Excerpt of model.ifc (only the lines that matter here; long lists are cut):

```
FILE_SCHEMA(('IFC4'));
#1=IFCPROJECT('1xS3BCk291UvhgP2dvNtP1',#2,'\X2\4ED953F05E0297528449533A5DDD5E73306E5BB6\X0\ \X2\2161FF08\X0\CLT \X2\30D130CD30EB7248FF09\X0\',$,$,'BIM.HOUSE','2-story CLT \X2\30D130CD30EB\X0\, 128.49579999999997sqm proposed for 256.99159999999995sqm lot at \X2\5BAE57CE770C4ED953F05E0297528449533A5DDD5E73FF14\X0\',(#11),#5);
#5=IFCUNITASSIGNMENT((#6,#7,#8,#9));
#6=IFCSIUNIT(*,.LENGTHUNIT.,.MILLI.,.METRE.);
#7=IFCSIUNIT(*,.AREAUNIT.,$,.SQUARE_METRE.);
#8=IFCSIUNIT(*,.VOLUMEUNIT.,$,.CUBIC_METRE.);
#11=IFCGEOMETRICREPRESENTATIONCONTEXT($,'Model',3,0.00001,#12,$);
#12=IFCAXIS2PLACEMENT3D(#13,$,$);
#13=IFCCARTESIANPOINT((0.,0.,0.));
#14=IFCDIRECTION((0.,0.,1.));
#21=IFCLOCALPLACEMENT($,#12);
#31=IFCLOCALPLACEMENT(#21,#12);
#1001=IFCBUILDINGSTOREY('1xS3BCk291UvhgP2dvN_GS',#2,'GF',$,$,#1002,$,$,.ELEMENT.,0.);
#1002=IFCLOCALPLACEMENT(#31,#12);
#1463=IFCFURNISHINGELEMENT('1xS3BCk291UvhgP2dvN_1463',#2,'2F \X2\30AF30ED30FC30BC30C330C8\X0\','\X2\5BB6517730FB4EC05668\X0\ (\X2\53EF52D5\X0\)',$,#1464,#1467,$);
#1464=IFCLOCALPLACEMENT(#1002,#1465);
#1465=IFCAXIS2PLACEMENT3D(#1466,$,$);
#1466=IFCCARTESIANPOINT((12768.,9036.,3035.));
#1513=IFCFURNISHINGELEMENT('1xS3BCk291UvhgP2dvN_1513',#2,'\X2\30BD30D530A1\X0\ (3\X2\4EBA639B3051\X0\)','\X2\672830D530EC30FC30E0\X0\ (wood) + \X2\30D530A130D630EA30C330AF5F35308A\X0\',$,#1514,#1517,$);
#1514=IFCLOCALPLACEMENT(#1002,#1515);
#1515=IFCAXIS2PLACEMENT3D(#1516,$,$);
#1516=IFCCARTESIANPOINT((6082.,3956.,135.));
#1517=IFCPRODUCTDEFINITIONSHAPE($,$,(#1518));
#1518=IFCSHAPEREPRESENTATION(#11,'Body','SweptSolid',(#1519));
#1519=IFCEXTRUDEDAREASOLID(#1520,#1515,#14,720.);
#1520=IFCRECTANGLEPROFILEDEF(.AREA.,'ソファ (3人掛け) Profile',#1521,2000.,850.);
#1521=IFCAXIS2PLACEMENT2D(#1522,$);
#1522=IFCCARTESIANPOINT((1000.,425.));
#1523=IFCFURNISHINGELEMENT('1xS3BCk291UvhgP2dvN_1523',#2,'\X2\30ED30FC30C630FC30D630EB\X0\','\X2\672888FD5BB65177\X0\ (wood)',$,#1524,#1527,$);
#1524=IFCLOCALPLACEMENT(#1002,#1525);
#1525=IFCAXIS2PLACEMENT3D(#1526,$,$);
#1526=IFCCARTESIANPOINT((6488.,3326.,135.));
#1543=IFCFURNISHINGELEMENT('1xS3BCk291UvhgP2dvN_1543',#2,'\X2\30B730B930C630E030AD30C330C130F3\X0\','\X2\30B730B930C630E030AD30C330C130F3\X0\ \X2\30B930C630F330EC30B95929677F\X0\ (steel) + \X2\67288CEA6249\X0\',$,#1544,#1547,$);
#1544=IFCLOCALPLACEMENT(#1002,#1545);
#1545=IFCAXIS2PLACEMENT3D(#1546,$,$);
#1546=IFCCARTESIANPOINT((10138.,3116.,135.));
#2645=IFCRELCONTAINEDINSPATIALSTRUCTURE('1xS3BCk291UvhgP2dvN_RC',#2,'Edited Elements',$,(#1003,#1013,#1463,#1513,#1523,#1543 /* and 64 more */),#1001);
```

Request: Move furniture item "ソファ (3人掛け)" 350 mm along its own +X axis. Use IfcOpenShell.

```python
import ifcopenshell
import ifcopenshell.api.geometry
import ifcopenshell.util.placement
import ifcopenshell.util.unit

model = ifcopenshell.open("model.ifc")
unit_scale = ifcopenshell.util.unit.calculate_unit_scale(model)

item = model.by_guid("1xS3BCk291UvhgP2dvN_1513")
matrix = ifcopenshell.util.placement.get_local_placement(item.ObjectPlacement)
matrix[:3, 3] += matrix[:3, 0] * 0.35 / unit_scale
ifcopenshell.api.geometry.edit_object_placement(model, product=item, matrix=matrix, is_si=False)

print(ifcopenshell.util.placement.get_local_placement(item.ObjectPlacement).round(3) + 0.0)

model.write("model_edited.ifc")
```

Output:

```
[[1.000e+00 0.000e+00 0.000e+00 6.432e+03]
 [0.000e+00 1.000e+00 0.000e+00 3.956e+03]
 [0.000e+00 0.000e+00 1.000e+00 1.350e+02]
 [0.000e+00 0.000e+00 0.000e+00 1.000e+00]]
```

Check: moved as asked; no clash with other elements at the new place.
